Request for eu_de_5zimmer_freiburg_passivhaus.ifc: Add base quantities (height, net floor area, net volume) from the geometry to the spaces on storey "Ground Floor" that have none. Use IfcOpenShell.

First a look at what the model holds.

```python
import ifcopenshell
import ifcopenshell.util.element
import ifcopenshell.util.unit

model = ifcopenshell.open("eu_de_5zimmer_freiburg_passivhaus.ifc")
print(model.schema)
for unit_type in ("LENGTHUNIT", "AREAUNIT", "VOLUMEUNIT"):
    print(unit_type, ifcopenshell.util.unit.calculate_unit_scale(model, unit_type))
storey = next(s for s in model.by_type("IfcBuildingStorey") if s.Name == "Ground Floor")
spaces = [e for e in ifcopenshell.util.element.get_decomposition(storey) if e.is_a("IfcSpace")]
for e in sorted(spaces, key=lambda e: e.id()):
    print(e.id(), e.is_a(), e.Name, list(ifcopenshell.util.element.get_psets(e, qtos_only=True)), sep=" | ")
```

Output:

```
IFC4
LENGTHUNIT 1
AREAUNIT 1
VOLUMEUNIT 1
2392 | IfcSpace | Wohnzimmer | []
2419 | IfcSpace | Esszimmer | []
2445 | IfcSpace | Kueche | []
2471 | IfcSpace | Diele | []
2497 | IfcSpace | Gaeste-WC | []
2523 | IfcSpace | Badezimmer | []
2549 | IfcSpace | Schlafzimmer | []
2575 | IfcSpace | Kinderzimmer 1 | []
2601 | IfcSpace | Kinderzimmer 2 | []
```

```python
import ifcopenshell
import ifcopenshell.api.pset
import ifcopenshell.geom
import ifcopenshell.util.element
import ifcopenshell.util.shape
import ifcopenshell.util.unit

model = ifcopenshell.open("eu_de_5zimmer_freiburg_passivhaus.ifc")
unit_scale = ifcopenshell.util.unit.calculate_unit_scale(model)
area_scale = ifcopenshell.util.unit.calculate_unit_scale(model, "AREAUNIT")
volume_scale = ifcopenshell.util.unit.calculate_unit_scale(model, "VOLUMEUNIT")
settings = ifcopenshell.geom.settings()

storey = next(s for s in model.by_type("IfcBuildingStorey") if s.Name == "Ground Floor")
spaces = [e for e in ifcopenshell.util.element.get_decomposition(storey) if e.is_a("IfcSpace")]

for e in sorted(spaces, key=lambda e: e.id()):
    if ifcopenshell.util.element.get_psets(e, qtos_only=True, should_inherit=False):
        continue
    # Geometry comes back in metres, in the element's own axes.
    shape = ifcopenshell.geom.create_shape(settings, e)
    values = {
        "Height": ifcopenshell.util.shape.get_z(shape.geometry) / unit_scale,
        "NetFloorArea": ifcopenshell.util.shape.get_footprint_area(shape.geometry) / area_scale,
        "NetVolume": ifcopenshell.util.shape.get_volume(shape.geometry) / volume_scale,
    }
    qto = ifcopenshell.api.pset.add_qto(model, product=e, name="Qto_SpaceBaseQuantities")
    ifcopenshell.api.pset.edit_qto(model, qto=qto, properties=values)
    print(e.id(), {k: round(v, 3) for k, v in values.items()})

model.write("eu_de_5zimmer_freiburg_passivhaus_rev.ifc")
```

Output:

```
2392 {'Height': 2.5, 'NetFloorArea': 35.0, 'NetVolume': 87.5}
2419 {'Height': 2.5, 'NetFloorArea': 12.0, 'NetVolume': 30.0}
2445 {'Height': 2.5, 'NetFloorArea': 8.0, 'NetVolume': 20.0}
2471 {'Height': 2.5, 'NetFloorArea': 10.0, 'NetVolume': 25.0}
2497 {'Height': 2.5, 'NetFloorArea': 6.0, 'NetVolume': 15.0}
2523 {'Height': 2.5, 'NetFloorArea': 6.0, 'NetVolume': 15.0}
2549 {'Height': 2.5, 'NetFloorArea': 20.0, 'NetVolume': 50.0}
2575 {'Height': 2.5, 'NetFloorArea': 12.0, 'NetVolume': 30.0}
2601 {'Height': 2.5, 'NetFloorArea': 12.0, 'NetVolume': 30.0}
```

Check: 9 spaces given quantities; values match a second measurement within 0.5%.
